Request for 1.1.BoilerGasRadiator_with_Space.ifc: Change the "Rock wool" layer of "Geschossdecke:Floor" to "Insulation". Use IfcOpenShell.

First a look at what the model holds.

```python
import ifcopenshell
import ifcopenshell.util.element

model = ifcopenshell.open("1.1.BoilerGasRadiator_with_Space.ifc")
print(model.schema)
for layer_set in model.by_type("IfcMaterialLayerSet"):
    if layer_set.LayerSetName == "Geschossdecke:Floor":
        for layer in layer_set.MaterialLayers:
            print(layer.id(), layer.Material and layer.Material.Name, layer.LayerThickness, sep=" | ")
        print(len(ifcopenshell.util.element.get_elements_by_material(model, layer_set)), "elements and types use it")
print(sorted(m.Name for m in model.by_type("IfcMaterial") if m.Name)[:60])
```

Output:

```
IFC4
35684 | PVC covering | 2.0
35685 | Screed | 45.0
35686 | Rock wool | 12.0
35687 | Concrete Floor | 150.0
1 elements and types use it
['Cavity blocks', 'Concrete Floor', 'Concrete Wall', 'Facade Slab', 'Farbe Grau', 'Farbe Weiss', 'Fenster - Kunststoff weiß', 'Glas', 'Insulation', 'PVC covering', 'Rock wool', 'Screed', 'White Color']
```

```python
import ifcopenshell
import ifcopenshell.api.material

model = ifcopenshell.open("1.1.BoilerGasRadiator_with_Space.ifc")

layer_set = next(s for s in model.by_type("IfcMaterialLayerSet") if s.LayerSetName == "Geschossdecke:Floor")
layer = next(l for l in layer_set.MaterialLayers if l.Material and l.Material.Name == "Rock wool")
material = next(m for m in model.by_type("IfcMaterial") if m.Name == "Insulation")

# Point this one layer at the other material; renaming the old one would change it everywhere.
ifcopenshell.api.material.edit_layer(model, layer=layer, attributes={}, material=material)

print([l.Material.Name if l.Material else None for l in layer_set.MaterialLayers])

model.write("1.1.BoilerGasRadiator_with_Space_edited.ifc")
```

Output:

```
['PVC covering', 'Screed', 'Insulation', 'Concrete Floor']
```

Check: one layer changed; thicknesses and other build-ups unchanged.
